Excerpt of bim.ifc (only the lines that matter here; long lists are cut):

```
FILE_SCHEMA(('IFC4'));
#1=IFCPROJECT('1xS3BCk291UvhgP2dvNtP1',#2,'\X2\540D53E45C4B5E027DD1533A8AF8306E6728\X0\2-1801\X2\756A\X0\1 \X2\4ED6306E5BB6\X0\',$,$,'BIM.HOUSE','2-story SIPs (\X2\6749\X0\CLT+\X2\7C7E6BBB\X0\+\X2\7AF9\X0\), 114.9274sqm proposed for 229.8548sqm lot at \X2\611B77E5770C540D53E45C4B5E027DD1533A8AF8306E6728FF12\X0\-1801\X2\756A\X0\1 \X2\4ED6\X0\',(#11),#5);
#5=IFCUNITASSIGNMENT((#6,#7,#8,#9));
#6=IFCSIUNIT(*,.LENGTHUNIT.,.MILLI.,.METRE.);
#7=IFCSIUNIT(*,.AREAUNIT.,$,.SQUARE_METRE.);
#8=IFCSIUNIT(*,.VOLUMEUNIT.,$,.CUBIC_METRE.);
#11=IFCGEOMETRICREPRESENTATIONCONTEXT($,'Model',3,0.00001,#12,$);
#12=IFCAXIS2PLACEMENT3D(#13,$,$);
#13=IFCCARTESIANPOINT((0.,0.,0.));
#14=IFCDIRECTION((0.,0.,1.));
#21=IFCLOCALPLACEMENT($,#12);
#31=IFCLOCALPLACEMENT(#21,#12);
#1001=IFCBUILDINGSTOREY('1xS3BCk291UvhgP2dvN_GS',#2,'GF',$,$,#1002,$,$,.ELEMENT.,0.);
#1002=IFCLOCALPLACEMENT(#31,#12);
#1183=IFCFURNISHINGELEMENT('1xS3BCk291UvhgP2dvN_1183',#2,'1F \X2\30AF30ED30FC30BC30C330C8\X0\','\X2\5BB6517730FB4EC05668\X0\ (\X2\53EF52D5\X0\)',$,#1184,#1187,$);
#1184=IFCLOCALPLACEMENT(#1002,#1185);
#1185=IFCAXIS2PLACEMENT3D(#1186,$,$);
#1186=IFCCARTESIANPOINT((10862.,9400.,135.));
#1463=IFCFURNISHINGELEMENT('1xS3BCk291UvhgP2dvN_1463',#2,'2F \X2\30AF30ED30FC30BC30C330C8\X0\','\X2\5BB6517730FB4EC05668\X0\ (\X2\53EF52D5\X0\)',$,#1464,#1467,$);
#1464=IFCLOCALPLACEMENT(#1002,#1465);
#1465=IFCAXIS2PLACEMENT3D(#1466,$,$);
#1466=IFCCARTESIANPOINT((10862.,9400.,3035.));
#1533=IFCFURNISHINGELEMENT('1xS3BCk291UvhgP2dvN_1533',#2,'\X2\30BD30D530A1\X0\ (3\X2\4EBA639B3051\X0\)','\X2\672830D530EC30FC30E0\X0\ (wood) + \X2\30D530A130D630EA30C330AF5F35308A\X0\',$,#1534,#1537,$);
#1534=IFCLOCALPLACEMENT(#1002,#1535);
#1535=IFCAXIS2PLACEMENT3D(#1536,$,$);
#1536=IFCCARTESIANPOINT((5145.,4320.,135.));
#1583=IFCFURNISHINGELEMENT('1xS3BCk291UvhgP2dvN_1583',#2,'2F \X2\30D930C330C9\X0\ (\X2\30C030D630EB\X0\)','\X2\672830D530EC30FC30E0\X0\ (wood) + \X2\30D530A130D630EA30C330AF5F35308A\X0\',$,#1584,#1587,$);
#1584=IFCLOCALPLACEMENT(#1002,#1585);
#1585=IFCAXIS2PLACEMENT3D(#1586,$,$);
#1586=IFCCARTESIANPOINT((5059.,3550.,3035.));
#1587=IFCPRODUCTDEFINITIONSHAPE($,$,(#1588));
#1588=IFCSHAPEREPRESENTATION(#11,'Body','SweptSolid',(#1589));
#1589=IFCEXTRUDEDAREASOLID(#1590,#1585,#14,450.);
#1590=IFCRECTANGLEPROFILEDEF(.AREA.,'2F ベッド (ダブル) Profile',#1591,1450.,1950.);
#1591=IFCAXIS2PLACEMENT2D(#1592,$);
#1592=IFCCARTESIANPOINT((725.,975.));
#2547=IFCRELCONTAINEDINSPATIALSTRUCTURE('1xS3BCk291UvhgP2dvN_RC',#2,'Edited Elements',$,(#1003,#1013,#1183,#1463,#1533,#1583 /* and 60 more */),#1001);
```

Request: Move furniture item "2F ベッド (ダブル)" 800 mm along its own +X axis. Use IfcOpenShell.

```python
import ifcopenshell
import ifcopenshell.api.geometry
import ifcopenshell.util.placement
import ifcopenshell.util.unit

model = ifcopenshell.open("bim.ifc")
unit_scale = ifcopenshell.util.unit.calculate_unit_scale(model)

item = model.by_guid("1xS3BCk291UvhgP2dvN_1583")
matrix = ifcopenshell.util.placement.get_local_placement(item.ObjectPlacement)
matrix[:3, 3] += matrix[:3, 0] * 0.8 / unit_scale
ifcopenshell.api.geometry.edit_object_placement(model, product=item, matrix=matrix, is_si=False)

print(ifcopenshell.util.placement.get_local_placement(item.ObjectPlacement).round(3) + 0.0)

model.write("bim-out.ifc")
```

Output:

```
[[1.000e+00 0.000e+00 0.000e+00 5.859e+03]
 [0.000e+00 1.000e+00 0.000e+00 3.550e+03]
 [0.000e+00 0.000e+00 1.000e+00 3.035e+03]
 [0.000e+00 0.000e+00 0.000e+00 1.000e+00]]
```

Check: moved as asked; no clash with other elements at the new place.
